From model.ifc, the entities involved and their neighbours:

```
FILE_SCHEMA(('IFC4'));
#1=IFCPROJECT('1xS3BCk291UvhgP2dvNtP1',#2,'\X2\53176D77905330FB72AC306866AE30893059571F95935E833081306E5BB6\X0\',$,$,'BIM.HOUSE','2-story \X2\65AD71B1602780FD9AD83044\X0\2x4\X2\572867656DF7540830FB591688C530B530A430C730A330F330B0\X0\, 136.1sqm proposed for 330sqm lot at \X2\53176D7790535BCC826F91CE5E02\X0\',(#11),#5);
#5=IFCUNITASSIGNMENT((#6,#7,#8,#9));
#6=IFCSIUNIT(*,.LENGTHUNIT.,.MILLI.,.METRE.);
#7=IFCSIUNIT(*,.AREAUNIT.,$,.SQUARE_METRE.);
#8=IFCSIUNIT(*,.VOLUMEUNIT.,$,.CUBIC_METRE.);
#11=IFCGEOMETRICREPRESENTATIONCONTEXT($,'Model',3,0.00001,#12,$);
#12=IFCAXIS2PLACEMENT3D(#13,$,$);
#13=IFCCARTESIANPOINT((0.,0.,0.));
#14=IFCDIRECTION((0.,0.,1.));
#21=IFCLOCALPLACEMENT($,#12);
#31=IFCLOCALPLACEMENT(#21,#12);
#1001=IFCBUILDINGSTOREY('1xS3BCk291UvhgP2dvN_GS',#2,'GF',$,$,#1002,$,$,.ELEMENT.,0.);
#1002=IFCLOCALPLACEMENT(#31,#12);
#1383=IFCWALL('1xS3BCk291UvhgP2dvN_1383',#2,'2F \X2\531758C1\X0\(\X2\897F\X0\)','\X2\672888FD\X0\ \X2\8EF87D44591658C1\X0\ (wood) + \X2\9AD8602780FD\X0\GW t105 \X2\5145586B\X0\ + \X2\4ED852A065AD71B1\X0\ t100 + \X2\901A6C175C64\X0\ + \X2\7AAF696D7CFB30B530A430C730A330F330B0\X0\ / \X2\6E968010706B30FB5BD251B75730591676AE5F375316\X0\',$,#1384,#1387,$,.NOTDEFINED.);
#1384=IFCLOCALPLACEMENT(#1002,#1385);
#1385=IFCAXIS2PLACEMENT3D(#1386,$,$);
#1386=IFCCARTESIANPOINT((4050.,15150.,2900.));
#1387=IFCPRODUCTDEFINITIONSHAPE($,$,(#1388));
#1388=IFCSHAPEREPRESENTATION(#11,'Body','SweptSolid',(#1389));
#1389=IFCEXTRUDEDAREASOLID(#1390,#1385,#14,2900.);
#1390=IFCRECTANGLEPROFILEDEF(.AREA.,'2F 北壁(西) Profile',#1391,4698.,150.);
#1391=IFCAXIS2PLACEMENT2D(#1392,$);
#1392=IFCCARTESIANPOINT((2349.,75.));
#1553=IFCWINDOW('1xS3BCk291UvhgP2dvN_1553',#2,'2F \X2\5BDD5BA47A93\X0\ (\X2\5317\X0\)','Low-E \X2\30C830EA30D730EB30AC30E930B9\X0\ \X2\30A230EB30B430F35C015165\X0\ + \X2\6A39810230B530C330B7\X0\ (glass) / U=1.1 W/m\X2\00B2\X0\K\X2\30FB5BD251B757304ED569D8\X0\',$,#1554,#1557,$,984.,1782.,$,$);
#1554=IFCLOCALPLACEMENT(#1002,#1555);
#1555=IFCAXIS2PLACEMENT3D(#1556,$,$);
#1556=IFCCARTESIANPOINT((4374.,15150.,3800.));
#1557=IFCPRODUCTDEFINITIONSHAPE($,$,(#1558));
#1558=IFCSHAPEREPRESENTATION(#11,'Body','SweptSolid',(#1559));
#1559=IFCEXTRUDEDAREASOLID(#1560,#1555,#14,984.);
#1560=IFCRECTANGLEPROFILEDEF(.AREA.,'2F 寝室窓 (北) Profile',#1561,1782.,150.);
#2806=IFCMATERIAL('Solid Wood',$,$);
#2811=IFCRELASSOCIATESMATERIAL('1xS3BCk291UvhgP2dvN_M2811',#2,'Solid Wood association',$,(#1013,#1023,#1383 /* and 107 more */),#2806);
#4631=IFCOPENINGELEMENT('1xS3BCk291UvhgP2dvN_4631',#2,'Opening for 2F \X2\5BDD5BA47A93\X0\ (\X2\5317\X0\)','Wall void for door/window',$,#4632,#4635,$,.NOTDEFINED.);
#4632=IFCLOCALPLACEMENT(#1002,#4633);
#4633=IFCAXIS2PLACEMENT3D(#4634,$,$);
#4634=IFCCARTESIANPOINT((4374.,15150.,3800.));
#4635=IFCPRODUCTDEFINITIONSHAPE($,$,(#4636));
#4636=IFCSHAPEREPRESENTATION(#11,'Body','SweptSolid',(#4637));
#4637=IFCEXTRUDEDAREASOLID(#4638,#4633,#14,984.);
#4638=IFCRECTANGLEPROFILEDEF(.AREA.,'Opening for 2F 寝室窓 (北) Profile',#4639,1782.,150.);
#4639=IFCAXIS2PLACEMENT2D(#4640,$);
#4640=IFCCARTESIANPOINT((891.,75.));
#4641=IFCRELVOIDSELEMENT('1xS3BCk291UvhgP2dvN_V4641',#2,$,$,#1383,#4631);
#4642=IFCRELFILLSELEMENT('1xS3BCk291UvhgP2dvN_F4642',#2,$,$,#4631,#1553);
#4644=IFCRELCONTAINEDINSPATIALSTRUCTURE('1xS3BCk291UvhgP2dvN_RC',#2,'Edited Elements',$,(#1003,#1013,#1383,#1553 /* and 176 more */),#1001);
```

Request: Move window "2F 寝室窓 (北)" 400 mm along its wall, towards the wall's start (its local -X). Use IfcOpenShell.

```python
import ifcopenshell
import ifcopenshell.api.geometry
import ifcopenshell.util.placement

model = ifcopenshell.open("model.ifc")

window = model.by_id(1553)
opening = window.FillsVoids[0].RelatingOpeningElement
wall = opening.VoidsElements[0].RelatingBuildingElement

wall_matrix = ifcopenshell.util.placement.get_local_placement(wall.ObjectPlacement)
shift = wall_matrix[:3, 0] * -400.0
before = ifcopenshell.util.placement.get_local_placement(window.ObjectPlacement)[:3, 3].copy()

# The window is not placed relative to its opening, so move both.
for product in (opening, window):
    matrix = ifcopenshell.util.placement.get_local_placement(product.ObjectPlacement)
    matrix[:3, 3] += shift
    ifcopenshell.api.geometry.edit_object_placement(model, product=product, matrix=matrix, is_si=False)

after = ifcopenshell.util.placement.get_local_placement(window.ObjectPlacement)[:3, 3]
print("window moved by", (after - before).round(3) + 0.0)

model.write("model_updated.ifc")
```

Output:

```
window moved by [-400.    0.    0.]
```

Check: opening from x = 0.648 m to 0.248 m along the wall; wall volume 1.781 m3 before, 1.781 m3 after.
